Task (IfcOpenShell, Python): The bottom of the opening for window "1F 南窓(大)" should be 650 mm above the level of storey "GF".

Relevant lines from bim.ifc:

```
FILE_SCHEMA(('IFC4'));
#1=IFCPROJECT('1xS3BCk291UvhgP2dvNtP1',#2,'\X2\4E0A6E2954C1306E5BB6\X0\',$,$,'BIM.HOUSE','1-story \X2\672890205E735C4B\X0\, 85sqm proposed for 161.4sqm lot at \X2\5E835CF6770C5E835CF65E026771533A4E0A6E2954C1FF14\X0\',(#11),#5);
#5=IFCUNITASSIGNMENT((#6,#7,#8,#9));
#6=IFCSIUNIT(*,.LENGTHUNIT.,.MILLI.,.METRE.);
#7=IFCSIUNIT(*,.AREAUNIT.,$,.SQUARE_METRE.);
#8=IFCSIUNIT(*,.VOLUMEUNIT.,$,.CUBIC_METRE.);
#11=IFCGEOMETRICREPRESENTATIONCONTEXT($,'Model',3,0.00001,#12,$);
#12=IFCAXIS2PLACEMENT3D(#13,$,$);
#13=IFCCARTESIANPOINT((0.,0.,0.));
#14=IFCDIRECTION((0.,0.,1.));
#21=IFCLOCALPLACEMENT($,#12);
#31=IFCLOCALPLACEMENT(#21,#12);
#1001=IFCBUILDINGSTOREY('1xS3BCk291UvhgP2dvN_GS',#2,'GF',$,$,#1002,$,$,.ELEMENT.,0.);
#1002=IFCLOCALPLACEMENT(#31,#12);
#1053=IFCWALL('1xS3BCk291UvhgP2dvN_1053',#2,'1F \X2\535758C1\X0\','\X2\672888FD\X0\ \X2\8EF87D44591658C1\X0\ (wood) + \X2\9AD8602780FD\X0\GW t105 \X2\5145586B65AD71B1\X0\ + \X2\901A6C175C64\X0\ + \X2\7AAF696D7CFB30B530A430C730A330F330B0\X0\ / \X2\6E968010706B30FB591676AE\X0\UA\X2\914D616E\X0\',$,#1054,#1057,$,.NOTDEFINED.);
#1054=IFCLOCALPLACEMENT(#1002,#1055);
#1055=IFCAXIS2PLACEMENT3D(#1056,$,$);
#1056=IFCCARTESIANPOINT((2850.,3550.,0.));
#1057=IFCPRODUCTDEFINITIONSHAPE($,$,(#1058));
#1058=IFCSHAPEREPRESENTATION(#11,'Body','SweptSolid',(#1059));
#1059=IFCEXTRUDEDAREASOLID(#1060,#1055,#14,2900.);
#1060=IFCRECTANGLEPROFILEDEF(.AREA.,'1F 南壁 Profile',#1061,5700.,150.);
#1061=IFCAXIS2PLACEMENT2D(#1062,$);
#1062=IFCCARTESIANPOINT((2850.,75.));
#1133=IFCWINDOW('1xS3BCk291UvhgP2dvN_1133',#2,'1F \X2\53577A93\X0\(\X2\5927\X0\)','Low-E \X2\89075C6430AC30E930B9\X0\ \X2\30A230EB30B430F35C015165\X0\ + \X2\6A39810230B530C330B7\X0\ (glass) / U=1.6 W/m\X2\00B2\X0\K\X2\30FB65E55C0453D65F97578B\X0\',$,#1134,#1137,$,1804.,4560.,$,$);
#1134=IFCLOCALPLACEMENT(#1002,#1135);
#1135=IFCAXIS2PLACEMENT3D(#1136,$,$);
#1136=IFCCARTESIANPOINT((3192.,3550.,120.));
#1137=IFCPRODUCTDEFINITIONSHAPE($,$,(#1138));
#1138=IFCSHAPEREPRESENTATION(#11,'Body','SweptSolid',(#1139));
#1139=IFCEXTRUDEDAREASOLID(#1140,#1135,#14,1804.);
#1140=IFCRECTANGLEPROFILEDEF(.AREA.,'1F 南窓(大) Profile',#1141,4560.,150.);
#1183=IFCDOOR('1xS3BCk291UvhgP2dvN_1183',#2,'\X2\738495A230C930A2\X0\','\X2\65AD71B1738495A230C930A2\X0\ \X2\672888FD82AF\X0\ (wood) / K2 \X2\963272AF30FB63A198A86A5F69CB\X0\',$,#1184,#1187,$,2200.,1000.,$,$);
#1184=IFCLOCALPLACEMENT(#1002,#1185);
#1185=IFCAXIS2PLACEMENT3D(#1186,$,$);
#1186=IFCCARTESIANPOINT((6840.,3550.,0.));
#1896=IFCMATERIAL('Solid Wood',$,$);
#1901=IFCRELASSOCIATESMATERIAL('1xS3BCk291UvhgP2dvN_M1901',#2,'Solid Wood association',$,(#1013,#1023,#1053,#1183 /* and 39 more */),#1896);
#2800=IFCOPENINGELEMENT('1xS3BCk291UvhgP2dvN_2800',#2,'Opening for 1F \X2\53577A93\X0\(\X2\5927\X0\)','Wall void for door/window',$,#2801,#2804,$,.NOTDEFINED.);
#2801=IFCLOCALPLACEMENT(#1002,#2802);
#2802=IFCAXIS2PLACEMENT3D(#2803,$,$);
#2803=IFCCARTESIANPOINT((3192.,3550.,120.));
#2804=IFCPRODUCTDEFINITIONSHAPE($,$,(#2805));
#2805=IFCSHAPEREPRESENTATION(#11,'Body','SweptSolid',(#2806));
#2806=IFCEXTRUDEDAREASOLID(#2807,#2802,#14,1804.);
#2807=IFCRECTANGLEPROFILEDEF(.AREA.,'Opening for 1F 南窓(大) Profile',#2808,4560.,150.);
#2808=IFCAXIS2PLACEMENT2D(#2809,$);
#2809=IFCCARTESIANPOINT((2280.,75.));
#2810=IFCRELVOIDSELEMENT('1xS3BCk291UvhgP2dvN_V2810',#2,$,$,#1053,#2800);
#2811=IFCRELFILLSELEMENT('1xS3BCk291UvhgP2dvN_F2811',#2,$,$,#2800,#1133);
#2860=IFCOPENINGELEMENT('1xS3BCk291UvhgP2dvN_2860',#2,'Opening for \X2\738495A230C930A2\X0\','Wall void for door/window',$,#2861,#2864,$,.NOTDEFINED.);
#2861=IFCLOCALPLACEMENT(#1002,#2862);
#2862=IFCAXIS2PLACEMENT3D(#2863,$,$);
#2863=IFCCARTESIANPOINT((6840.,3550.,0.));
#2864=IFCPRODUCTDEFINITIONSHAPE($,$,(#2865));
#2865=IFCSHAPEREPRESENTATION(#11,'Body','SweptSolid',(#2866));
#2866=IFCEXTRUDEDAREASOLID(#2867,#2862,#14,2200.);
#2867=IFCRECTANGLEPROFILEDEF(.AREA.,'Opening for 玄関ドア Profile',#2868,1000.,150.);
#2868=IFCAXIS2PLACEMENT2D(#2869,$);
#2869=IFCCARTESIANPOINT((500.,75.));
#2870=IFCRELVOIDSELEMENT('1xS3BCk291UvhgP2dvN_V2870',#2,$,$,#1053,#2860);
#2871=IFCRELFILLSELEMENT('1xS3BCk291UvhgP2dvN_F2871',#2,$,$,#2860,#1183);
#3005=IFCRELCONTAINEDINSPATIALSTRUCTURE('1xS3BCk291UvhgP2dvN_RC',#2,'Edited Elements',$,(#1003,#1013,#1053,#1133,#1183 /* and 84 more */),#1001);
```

```python
import numpy as np
import ifcopenshell
import ifcopenshell.api.geometry
import ifcopenshell.geom
import ifcopenshell.util.element
import ifcopenshell.util.placement
import ifcopenshell.util.shape
import ifcopenshell.util.unit

model = ifcopenshell.open("bim.ifc")
unit_scale = ifcopenshell.util.unit.calculate_unit_scale(model)

window = model.by_guid("1xS3BCk291UvhgP2dvN_1133")
opening = window.FillsVoids[0].RelatingOpeningElement
storey = ifcopenshell.util.element.get_container(window, ifc_class="IfcBuildingStorey")
level = ifcopenshell.util.placement.get_local_placement(storey.ObjectPlacement)[2, 3]

# The opening's origin need not be at the sill, so measure its lowest point.
shape = ifcopenshell.geom.create_shape(ifcopenshell.geom.settings(), opening)
bottom = ifcopenshell.util.shape.get_shape_bottom_elevation(shape, shape.geometry) / unit_scale
dz = level + 650.0 - bottom

shift = np.array([0.0, 0.0, dz])
# The window is not placed relative to its opening, so move both.
for product in (opening, window):
    matrix = ifcopenshell.util.placement.get_local_placement(product.ObjectPlacement)
    matrix[:3, 3] += shift
    ifcopenshell.api.geometry.edit_object_placement(model, product=product, matrix=matrix, is_si=False)

print(f"moved by {dz * unit_scale:+.3f} m")

model.write("bim_updated.ifc")
```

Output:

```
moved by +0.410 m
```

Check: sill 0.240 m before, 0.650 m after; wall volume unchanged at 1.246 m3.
